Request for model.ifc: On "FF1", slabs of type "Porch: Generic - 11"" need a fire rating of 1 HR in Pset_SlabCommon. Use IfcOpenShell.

First a look at what the model holds.

```python
import ifcopenshell
import ifcopenshell.util.element

model = ifcopenshell.open("model.ifc")
print(model.schema)
storey = next(s for s in model.by_type("IfcBuildingStorey") if s.Name == "FF1")
slabs = [e for e in ifcopenshell.util.element.get_decomposition(storey) if e.is_a("IfcSlab")]
seen = {}
for e in slabs:
    element_type = ifcopenshell.util.element.get_type(e)
    key = (element_type.Name if element_type != e and element_type else None, ifcopenshell.util.element.get_pset(e, "Pset_SlabCommon", "FireRating"))
    seen[key] = seen.get(key, 0) + 1
for (name, value), count in sorted(seen.items(), key=str):
    print(count, "x", name, "|", value)
```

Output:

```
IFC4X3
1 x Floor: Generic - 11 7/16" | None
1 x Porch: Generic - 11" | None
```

```python
import ifcopenshell
import ifcopenshell.api.pset
import ifcopenshell.util.element

model = ifcopenshell.open("model.ifc")

storey = next(s for s in model.by_type("IfcBuildingStorey") if s.Name == "FF1")
slabs = [e for e in ifcopenshell.util.element.get_decomposition(storey) if e.is_a("IfcSlab")]

count = 0
for e in slabs:
    element_type = ifcopenshell.util.element.get_type(e)
    if element_type in (None, e) or element_type.Name != 'Porch: Generic - 11"':
        continue
    # add_pset returns the element's existing set when there is one.
    pset = ifcopenshell.api.pset.add_pset(model, product=e, name="Pset_SlabCommon")
    ifcopenshell.api.pset.edit_pset(model, pset=pset, properties={"FireRating": "1 HR"})
    count += 1

print(count, "slabs updated")

model.write("model_v2.ifc")
```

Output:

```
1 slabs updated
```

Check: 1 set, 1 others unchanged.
